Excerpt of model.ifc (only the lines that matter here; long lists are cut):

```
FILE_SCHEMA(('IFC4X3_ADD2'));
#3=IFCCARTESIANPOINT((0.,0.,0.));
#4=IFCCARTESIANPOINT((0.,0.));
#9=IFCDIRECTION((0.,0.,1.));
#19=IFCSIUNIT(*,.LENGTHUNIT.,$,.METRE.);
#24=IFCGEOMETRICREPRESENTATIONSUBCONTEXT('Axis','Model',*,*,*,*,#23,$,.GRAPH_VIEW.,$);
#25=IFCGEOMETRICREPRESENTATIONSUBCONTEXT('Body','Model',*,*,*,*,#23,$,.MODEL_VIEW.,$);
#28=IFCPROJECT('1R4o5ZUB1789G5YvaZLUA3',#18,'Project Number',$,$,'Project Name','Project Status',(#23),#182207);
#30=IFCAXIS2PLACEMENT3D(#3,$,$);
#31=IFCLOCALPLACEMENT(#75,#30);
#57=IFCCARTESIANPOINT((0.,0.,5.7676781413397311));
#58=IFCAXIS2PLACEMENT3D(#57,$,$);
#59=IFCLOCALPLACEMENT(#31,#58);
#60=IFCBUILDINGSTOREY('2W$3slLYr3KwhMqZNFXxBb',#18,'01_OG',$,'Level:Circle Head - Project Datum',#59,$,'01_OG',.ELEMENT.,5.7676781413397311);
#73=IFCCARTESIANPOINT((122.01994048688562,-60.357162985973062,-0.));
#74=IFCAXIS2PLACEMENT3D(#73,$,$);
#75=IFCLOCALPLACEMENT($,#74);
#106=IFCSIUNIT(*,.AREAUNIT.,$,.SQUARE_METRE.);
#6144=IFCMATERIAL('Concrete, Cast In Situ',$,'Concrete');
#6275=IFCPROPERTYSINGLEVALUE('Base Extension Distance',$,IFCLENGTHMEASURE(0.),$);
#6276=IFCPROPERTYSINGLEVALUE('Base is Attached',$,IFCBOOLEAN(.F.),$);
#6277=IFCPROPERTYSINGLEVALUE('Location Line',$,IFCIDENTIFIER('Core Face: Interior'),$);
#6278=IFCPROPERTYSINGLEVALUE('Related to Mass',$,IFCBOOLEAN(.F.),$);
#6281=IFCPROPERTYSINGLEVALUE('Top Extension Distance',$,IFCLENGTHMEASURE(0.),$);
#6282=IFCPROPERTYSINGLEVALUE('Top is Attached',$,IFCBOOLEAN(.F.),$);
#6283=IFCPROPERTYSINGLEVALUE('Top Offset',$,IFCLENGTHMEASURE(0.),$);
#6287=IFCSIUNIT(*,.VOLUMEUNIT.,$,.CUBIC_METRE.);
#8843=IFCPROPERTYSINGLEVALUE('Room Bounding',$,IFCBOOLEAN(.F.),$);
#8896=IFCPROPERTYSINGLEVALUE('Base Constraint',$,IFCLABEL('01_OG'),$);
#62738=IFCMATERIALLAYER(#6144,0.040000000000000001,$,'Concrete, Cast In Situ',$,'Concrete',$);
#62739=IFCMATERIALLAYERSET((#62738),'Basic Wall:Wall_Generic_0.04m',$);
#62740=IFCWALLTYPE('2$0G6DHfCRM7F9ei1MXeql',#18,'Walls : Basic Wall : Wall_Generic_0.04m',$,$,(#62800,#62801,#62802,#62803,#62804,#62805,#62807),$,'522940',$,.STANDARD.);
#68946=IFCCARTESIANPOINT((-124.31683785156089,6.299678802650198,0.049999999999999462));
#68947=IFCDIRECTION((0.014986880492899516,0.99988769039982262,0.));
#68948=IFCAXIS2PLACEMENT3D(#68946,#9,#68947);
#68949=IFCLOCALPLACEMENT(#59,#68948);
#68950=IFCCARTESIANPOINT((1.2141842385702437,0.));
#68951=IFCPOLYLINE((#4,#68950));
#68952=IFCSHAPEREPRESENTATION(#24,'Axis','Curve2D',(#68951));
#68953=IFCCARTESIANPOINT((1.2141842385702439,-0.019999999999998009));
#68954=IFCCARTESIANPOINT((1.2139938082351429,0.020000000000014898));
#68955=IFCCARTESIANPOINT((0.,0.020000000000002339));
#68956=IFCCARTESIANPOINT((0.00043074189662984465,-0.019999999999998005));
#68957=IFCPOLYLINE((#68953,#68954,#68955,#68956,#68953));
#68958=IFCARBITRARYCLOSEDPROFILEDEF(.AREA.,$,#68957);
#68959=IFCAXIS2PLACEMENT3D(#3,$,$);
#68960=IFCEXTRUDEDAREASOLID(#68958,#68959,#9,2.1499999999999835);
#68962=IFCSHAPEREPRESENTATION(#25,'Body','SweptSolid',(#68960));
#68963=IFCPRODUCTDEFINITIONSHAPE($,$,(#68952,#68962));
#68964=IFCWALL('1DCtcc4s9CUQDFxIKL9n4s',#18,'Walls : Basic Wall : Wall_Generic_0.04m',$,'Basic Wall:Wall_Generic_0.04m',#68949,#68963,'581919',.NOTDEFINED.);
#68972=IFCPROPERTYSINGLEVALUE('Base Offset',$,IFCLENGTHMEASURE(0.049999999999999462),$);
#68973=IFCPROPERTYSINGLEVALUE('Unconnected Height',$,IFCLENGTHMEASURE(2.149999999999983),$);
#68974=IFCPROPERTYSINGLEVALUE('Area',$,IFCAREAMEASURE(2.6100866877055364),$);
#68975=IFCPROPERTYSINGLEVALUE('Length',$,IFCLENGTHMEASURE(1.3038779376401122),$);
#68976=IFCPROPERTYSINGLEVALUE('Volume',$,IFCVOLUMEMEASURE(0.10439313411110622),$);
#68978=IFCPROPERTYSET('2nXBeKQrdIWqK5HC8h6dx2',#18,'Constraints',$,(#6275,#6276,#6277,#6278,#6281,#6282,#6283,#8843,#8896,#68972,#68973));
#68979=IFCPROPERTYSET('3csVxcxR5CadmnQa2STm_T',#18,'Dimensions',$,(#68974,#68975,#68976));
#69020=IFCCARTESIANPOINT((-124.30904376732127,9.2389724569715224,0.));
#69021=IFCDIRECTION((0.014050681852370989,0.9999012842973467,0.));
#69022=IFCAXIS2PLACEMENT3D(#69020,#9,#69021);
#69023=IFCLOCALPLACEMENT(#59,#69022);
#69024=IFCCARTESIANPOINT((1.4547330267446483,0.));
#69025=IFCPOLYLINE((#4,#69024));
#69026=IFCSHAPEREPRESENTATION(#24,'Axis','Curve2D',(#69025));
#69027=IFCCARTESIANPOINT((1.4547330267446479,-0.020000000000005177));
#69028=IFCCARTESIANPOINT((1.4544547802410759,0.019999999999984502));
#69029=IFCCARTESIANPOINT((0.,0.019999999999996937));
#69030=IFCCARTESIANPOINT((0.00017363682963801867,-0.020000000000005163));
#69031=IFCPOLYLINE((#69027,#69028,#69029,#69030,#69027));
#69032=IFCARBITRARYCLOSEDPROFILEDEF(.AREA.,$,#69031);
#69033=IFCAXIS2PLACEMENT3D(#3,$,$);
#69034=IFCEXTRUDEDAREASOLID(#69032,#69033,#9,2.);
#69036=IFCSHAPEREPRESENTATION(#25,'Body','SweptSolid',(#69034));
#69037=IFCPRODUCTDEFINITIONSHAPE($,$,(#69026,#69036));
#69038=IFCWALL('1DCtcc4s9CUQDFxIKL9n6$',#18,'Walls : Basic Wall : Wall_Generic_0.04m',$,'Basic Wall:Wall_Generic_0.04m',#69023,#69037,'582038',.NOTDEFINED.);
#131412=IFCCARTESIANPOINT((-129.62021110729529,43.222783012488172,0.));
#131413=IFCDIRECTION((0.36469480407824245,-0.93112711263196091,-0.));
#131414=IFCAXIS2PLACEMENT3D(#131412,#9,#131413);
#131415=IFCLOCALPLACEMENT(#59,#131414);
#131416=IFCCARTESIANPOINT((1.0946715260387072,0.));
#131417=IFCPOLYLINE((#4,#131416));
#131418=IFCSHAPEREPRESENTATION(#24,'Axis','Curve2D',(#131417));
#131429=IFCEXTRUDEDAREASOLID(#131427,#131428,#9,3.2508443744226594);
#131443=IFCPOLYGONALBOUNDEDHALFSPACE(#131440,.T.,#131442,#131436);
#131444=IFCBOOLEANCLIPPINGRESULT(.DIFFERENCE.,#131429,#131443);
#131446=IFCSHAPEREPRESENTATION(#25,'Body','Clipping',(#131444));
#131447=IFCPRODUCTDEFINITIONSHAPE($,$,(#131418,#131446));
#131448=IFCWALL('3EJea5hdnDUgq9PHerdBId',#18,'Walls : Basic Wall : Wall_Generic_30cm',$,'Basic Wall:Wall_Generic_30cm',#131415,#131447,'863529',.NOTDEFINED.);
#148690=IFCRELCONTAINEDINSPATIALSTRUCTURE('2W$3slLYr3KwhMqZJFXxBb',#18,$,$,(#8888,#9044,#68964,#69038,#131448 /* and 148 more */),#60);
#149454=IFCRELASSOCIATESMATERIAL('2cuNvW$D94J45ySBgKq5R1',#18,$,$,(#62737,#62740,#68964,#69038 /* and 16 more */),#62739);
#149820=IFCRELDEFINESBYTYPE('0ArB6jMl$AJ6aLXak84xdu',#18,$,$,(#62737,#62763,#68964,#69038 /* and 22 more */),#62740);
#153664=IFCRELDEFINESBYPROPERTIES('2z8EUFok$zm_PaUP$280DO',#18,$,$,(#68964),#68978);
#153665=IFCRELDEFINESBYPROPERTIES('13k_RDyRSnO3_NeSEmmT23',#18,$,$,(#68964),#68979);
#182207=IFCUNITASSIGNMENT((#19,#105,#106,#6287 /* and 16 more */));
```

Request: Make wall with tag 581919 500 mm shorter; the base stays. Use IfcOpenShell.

```python
import ifcopenshell
import ifcopenshell.api.pset
import ifcopenshell.geom
import ifcopenshell.util.element
import ifcopenshell.util.representation
import ifcopenshell.util.shape
import ifcopenshell.util.unit

model = ifcopenshell.open("model.ifc")
area_scale = ifcopenshell.util.unit.calculate_unit_scale(model, "AREAUNIT")
volume_scale = ifcopenshell.util.unit.calculate_unit_scale(model, "VOLUMEUNIT")
settings = ifcopenshell.geom.settings()


def volume(element):
    """Net volume in cubic metres, openings subtracted."""
    shape = ifcopenshell.geom.create_shape(settings, element)
    return ifcopenshell.util.shape.get_volume(shape.geometry)


wall = model.by_id(68964)
before = volume(wall)

body = ifcopenshell.util.representation.get_representation(wall, "Model", "Body")
solid = body.Items[0]
old_height = solid.Depth
solid.Depth -= 0.5
after = volume(wall)
thickness = 0.04  # wall thickness in metres

# Update the stored height, areas and volumes.
pset = model.by_id(ifcopenshell.util.element.get_pset(wall, "Constraints", should_inherit=False)["id"])
ifcopenshell.api.pset.edit_pset(model, pset=pset, properties={
    "Unconnected Height": model.create_entity("IfcLengthMeasure", solid.Depth),
})
pset = model.by_id(ifcopenshell.util.element.get_pset(wall, "Dimensions", should_inherit=False)["id"])
ifcopenshell.api.pset.edit_pset(model, pset=pset, properties={
    "Area": model.create_entity("IfcAreaMeasure", after / thickness / area_scale),
    "Volume": model.create_entity("IfcVolumeMeasure", after / volume_scale),
})

print(f"height {old_height:g} -> {solid.Depth:g}, volume {before:.3f} -> {after:.3f} m3")

model.write("model_rev.ifc")
```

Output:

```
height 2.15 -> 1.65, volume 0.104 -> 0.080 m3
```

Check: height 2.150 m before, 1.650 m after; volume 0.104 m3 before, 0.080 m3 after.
